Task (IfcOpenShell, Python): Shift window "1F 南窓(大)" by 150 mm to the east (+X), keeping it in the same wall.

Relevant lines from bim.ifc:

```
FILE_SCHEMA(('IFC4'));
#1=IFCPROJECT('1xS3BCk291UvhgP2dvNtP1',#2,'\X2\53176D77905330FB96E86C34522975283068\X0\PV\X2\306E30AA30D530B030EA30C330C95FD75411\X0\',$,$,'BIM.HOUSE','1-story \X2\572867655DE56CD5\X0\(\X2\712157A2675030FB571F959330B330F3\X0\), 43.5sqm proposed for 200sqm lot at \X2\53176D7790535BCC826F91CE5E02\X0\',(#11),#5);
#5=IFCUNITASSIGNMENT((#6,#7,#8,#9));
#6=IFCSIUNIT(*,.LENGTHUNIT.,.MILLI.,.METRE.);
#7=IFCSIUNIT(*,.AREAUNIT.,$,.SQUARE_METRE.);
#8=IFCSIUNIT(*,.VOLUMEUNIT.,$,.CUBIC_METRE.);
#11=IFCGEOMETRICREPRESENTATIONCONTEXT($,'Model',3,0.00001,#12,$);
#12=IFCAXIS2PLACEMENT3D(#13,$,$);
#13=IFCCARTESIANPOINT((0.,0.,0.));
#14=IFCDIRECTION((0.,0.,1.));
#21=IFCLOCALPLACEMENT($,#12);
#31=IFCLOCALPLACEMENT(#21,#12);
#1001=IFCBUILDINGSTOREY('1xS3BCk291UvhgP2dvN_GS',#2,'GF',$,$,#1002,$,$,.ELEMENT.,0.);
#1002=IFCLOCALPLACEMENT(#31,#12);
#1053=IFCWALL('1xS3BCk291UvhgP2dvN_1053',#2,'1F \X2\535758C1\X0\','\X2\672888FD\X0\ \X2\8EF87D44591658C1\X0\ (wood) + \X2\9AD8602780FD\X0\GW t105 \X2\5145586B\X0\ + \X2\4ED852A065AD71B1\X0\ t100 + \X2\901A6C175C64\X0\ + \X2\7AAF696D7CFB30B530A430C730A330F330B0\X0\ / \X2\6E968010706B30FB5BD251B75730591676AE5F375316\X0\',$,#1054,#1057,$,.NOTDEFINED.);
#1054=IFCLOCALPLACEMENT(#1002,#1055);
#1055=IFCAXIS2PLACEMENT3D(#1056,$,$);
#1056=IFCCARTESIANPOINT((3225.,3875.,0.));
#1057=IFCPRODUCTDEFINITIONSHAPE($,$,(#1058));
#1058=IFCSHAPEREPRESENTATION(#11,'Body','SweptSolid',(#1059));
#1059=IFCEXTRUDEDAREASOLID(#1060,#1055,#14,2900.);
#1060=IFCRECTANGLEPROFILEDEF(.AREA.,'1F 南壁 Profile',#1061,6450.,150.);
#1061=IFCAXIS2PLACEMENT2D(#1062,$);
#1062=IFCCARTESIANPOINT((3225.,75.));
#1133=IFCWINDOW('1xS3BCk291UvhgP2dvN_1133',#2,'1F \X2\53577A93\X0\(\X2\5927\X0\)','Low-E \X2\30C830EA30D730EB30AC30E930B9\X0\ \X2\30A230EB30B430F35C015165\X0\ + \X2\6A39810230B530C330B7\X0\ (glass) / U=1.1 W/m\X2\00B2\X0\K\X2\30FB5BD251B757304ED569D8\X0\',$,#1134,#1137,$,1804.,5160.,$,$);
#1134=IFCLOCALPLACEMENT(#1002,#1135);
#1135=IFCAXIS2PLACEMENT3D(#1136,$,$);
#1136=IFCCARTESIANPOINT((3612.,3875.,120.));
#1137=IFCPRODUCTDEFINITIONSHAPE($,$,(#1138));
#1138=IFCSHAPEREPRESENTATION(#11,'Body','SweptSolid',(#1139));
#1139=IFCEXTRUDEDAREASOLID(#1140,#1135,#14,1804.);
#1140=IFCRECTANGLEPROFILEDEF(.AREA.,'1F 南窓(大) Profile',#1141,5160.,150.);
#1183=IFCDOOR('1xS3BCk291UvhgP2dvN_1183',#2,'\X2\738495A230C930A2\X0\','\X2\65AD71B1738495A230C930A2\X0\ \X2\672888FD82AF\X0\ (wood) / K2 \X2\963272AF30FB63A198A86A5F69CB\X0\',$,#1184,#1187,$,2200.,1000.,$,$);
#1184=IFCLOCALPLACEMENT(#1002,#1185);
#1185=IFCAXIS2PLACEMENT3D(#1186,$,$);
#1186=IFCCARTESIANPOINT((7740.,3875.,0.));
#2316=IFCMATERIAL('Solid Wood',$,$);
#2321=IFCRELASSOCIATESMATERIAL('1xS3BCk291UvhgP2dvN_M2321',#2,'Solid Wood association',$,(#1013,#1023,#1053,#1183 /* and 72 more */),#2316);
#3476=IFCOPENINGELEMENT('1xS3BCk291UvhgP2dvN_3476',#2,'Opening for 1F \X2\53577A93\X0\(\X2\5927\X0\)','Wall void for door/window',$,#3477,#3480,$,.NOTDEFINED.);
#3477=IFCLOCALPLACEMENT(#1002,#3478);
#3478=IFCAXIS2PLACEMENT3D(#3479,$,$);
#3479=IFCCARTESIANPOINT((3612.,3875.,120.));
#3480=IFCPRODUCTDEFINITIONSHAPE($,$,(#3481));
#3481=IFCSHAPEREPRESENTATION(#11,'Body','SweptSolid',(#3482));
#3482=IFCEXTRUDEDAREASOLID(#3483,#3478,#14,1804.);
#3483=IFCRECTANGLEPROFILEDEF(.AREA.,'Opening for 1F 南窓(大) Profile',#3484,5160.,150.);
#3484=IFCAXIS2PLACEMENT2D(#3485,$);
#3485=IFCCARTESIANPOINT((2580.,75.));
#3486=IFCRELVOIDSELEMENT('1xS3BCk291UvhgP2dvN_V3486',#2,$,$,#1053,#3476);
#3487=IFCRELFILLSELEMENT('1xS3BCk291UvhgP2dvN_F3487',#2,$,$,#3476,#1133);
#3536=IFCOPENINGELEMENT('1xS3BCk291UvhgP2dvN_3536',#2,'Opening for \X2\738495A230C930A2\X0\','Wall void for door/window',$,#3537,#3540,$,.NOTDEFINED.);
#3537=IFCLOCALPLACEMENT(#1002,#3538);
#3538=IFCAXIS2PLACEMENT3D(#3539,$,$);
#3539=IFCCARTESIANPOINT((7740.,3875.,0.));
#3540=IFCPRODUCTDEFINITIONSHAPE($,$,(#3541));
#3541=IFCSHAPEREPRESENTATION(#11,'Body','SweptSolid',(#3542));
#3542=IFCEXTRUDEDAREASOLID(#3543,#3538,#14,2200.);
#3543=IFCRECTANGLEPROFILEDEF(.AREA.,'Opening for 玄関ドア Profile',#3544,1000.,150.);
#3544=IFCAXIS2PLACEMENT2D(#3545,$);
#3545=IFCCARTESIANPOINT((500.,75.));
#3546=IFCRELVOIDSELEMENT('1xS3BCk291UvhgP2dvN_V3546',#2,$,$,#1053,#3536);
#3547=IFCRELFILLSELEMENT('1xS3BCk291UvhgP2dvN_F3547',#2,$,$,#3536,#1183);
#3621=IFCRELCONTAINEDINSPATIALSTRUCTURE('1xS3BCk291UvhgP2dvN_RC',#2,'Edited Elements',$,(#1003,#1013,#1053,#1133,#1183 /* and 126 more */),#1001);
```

```python
import ifcopenshell
import ifcopenshell.api.geometry
import ifcopenshell.util.placement
import ifcopenshell.util.unit

model = ifcopenshell.open("bim.ifc")
unit_scale = ifcopenshell.util.unit.calculate_unit_scale(model)

window = model.by_id(1133)
opening = window.FillsVoids[0].RelatingOpeningElement
wall = opening.VoidsElements[0].RelatingBuildingElement

wall_matrix = ifcopenshell.util.placement.get_local_placement(wall.ObjectPlacement)
shift = wall_matrix[:3, 0] * 0.15 / unit_scale
before = ifcopenshell.util.placement.get_local_placement(window.ObjectPlacement)[:3, 3].copy()

# The window is not placed relative to its opening, so move both.
for product in (opening, window):
    matrix = ifcopenshell.util.placement.get_local_placement(product.ObjectPlacement)
    matrix[:3, 3] += shift
    ifcopenshell.api.geometry.edit_object_placement(model, product=product, matrix=matrix, is_si=False)

after = ifcopenshell.util.placement.get_local_placement(window.ObjectPlacement)[:3, 3]
print("window moved by", (after - before).round(3) + 0.0)

model.write("bim-out.ifc")
```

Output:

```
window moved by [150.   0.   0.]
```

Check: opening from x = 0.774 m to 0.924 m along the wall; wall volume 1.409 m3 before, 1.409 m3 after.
